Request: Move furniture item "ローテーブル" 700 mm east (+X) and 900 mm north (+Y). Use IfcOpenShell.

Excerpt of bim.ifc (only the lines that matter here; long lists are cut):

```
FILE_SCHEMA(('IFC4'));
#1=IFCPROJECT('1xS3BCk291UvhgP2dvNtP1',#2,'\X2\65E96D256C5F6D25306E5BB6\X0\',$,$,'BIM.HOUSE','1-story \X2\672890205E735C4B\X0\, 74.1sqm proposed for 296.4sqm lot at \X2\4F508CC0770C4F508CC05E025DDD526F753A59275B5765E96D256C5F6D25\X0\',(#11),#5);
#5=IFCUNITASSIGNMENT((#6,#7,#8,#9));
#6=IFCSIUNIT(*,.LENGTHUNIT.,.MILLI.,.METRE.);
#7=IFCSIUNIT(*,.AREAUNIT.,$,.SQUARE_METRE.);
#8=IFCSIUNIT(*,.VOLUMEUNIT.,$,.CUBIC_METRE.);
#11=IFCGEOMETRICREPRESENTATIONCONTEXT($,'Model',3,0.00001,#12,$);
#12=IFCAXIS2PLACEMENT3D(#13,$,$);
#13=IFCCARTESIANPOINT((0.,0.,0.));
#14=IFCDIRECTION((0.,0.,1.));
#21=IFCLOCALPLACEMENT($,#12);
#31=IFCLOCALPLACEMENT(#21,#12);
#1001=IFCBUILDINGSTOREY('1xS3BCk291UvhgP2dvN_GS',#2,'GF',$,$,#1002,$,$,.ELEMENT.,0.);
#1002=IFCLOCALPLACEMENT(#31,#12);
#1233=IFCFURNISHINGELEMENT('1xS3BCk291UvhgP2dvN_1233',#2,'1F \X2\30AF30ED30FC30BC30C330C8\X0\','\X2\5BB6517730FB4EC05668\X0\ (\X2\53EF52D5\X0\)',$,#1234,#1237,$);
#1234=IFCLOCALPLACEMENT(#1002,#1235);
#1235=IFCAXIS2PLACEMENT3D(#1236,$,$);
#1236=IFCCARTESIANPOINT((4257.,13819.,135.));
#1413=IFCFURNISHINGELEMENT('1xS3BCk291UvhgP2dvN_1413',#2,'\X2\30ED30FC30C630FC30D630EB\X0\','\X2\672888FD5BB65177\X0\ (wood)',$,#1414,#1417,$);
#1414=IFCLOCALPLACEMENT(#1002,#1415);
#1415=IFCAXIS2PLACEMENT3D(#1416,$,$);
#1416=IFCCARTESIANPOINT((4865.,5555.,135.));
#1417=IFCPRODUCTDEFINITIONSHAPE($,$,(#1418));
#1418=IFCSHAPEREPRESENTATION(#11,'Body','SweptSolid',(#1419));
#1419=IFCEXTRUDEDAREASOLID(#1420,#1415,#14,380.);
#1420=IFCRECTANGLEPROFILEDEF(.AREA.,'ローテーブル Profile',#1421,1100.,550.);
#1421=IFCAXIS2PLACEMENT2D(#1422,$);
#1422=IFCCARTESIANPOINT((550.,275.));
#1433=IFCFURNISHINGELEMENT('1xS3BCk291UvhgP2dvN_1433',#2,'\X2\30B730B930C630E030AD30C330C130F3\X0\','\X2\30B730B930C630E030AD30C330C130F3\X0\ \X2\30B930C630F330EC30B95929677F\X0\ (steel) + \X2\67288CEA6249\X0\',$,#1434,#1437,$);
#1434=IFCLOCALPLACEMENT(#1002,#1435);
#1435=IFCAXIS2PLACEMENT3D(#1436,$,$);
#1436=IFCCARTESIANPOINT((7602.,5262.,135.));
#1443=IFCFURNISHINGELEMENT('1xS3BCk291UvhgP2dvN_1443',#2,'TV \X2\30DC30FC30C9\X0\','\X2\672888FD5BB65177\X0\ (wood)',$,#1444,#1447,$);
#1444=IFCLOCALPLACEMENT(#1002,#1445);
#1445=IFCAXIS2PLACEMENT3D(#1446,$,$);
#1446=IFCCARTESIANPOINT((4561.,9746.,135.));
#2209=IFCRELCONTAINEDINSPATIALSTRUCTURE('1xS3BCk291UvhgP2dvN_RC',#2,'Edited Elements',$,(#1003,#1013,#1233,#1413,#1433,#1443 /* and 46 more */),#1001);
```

```python
import ifcopenshell
import ifcopenshell.api.geometry
import ifcopenshell.util.placement

model = ifcopenshell.open("bim.ifc")

item = model.by_guid("1xS3BCk291UvhgP2dvN_1413")
matrix = ifcopenshell.util.placement.get_local_placement(item.ObjectPlacement)
matrix[0, 3] += 700.0
matrix[1, 3] += 900.0
ifcopenshell.api.geometry.edit_object_placement(model, product=item, matrix=matrix, is_si=False)

print(ifcopenshell.util.placement.get_local_placement(item.ObjectPlacement).round(3) + 0.0)

model.write("bim_v2.ifc")
```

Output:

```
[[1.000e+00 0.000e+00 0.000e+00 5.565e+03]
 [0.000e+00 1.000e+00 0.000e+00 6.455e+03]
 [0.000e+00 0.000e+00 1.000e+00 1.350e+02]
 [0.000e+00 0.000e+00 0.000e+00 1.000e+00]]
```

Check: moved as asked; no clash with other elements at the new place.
